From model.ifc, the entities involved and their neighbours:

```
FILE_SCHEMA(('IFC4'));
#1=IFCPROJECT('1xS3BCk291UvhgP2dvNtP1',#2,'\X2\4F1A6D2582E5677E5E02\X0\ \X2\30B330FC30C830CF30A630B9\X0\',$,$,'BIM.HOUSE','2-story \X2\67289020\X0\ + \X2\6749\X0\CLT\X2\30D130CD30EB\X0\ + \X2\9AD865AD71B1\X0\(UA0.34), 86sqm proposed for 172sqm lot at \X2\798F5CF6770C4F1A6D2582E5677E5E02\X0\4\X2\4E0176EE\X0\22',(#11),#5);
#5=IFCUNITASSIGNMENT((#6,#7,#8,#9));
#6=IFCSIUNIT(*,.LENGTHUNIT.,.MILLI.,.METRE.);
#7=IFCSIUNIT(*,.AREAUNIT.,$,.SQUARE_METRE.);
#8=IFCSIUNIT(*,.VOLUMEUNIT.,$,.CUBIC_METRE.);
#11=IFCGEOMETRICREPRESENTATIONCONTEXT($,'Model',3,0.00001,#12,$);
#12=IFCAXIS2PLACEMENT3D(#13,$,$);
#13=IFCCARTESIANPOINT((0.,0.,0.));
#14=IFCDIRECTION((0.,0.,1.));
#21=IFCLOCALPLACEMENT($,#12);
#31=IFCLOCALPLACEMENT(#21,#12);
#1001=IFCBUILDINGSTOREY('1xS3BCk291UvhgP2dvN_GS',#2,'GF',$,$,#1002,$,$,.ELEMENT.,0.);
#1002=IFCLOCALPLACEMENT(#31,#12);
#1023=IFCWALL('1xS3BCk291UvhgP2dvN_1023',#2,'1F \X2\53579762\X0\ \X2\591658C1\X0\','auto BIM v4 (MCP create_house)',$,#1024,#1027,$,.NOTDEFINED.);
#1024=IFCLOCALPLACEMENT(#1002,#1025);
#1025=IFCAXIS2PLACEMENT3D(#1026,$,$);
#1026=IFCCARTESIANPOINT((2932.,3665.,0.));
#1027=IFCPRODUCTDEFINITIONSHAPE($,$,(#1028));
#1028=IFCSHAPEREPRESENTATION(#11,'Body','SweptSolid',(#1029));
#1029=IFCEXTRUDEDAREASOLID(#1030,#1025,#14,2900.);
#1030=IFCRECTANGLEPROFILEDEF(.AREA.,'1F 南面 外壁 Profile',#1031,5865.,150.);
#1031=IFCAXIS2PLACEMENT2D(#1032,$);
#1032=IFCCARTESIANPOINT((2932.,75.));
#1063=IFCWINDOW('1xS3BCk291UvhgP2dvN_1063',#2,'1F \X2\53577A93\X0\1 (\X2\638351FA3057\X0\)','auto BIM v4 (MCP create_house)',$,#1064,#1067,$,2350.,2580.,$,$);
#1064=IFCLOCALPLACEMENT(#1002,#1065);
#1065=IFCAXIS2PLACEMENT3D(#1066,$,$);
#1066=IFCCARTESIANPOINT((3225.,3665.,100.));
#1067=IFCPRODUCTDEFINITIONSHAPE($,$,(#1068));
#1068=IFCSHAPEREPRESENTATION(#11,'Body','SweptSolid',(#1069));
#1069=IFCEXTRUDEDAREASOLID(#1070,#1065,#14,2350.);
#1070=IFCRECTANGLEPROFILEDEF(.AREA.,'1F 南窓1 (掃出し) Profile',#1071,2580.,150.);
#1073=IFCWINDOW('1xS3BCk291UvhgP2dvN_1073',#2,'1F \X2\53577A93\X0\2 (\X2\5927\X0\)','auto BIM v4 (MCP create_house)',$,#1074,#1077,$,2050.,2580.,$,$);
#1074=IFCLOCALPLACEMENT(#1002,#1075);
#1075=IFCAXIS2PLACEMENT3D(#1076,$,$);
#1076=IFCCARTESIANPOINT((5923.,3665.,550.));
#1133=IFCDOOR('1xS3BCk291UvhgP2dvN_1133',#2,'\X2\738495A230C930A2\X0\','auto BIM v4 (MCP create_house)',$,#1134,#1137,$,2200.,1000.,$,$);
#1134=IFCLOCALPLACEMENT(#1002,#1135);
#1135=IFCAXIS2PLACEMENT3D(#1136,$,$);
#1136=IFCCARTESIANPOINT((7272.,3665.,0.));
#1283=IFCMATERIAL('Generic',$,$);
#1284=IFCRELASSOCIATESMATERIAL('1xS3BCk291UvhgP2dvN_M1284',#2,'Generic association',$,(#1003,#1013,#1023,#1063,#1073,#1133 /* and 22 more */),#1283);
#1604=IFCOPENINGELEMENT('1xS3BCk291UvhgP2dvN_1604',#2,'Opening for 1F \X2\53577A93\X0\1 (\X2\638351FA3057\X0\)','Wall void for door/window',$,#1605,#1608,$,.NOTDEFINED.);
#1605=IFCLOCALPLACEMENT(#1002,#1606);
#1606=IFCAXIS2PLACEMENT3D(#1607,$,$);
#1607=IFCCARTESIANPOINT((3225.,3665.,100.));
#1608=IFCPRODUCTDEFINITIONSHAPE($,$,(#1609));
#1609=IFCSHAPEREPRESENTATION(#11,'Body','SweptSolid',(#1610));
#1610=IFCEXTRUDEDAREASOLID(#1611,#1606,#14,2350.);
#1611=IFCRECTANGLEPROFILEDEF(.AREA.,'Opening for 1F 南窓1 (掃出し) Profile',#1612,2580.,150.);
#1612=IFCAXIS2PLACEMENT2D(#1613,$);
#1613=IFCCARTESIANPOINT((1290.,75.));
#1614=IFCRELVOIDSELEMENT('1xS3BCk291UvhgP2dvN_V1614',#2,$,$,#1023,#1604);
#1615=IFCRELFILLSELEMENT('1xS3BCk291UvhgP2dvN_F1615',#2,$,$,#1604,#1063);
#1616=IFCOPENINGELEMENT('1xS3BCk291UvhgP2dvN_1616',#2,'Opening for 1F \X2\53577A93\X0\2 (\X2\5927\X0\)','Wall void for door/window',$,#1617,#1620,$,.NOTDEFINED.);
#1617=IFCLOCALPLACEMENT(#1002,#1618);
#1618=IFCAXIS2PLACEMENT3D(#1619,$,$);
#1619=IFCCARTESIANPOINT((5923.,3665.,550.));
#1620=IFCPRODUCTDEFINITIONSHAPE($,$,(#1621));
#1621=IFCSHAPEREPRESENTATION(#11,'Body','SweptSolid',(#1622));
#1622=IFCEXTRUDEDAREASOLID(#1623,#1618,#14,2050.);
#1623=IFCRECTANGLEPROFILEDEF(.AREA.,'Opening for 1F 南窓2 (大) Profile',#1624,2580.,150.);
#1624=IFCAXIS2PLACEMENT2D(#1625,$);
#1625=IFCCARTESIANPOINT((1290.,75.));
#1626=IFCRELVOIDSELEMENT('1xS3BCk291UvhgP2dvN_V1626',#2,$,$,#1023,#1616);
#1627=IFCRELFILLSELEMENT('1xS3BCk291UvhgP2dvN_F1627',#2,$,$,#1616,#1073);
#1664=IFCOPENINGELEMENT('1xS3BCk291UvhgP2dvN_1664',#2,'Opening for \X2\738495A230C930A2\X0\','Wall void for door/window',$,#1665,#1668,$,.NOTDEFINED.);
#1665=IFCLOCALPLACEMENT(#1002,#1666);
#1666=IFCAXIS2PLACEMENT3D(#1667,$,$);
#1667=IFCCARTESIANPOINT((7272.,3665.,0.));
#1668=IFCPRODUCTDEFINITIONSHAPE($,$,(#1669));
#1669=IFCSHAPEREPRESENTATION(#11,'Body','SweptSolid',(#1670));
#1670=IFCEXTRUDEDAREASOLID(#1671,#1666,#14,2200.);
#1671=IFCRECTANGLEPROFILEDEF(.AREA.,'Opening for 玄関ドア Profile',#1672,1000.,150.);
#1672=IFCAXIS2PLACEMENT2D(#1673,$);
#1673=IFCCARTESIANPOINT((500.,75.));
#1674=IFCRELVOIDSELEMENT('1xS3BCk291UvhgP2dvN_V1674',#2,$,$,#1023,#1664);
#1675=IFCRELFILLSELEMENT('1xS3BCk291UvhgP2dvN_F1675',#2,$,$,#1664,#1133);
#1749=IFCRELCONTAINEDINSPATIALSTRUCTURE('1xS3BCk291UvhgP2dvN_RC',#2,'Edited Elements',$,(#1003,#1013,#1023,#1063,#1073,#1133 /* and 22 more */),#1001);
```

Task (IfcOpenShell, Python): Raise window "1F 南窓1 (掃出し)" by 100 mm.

```python
import numpy as np
import ifcopenshell
import ifcopenshell.api.geometry
import ifcopenshell.util.placement
import ifcopenshell.util.unit

model = ifcopenshell.open("model.ifc")
unit_scale = ifcopenshell.util.unit.calculate_unit_scale(model)

window = model.by_guid("1xS3BCk291UvhgP2dvN_1063")
opening = window.FillsVoids[0].RelatingOpeningElement
dz = 0.1 / unit_scale

shift = np.array([0.0, 0.0, dz])
# The window is not placed relative to its opening, so move both.
for product in (opening, window):
    matrix = ifcopenshell.util.placement.get_local_placement(product.ObjectPlacement)
    matrix[:3, 3] += shift
    ifcopenshell.api.geometry.edit_object_placement(model, product=product, matrix=matrix, is_si=False)

print(f"moved by {dz * unit_scale:+.3f} m")

model.write("model-out.ifc")
```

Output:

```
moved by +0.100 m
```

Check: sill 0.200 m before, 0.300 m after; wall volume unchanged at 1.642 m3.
